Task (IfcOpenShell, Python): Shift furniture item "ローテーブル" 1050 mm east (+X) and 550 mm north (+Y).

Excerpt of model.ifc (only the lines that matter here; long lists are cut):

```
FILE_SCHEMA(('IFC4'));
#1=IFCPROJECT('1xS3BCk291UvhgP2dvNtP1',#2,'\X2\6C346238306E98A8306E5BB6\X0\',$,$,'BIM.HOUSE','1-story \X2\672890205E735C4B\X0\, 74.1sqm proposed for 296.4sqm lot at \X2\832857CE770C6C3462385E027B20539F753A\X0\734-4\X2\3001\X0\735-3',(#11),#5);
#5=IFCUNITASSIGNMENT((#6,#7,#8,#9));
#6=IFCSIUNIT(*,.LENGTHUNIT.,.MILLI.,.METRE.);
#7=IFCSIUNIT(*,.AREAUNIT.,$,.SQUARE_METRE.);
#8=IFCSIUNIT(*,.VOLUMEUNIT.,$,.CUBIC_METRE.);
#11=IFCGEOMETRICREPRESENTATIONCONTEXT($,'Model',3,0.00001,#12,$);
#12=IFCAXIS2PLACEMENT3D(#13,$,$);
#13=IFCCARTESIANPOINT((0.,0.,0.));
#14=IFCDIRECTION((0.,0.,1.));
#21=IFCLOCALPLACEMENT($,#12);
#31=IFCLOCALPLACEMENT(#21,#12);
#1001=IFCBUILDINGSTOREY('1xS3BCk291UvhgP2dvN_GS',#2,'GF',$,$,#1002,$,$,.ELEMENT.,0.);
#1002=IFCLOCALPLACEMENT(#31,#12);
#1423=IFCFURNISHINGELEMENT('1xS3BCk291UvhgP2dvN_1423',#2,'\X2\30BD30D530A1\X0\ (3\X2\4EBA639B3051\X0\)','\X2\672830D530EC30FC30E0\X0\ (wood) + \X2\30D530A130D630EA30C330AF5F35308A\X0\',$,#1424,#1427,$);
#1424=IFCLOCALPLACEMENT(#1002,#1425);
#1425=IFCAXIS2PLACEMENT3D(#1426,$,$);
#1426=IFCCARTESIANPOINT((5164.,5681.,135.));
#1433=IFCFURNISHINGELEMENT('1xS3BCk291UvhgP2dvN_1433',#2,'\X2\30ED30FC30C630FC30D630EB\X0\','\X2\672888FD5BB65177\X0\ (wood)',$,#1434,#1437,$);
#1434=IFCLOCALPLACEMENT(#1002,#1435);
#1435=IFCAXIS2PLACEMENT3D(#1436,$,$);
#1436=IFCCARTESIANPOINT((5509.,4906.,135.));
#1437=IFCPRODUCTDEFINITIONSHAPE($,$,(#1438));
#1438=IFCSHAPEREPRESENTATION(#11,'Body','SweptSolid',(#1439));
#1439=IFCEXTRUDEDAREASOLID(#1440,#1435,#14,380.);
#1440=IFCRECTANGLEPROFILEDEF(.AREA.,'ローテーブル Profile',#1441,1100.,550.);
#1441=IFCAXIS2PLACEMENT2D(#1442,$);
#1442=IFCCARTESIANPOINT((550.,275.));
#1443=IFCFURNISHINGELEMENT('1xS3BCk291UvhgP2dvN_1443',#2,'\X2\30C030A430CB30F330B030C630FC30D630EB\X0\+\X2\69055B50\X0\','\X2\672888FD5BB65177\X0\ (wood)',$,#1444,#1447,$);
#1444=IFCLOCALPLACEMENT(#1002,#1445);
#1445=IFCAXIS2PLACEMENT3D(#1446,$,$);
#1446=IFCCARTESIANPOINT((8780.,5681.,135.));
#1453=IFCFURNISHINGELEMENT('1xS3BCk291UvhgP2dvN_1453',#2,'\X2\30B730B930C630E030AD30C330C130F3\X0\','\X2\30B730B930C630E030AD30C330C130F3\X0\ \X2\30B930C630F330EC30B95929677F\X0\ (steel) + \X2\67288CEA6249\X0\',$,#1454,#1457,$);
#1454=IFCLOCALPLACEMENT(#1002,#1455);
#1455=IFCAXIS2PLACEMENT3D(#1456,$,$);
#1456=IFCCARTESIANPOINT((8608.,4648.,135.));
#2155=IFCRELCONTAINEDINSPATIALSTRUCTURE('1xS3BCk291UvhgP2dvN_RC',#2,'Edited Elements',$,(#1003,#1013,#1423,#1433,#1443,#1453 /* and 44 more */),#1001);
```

```python
import ifcopenshell
import ifcopenshell.api.geometry
import ifcopenshell.util.placement

model = ifcopenshell.open("model.ifc")

item = model.by_id(1433)
matrix = ifcopenshell.util.placement.get_local_placement(item.ObjectPlacement)
matrix[0, 3] += 1050.0
matrix[1, 3] += 550.0
ifcopenshell.api.geometry.edit_object_placement(model, product=item, matrix=matrix, is_si=False)

print(ifcopenshell.util.placement.get_local_placement(item.ObjectPlacement).round(3) + 0.0)

model.write("model_edited.ifc")
```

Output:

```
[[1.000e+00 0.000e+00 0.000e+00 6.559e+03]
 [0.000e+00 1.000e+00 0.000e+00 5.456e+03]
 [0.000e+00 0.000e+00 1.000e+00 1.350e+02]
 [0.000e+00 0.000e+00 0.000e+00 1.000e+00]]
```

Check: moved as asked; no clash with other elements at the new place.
